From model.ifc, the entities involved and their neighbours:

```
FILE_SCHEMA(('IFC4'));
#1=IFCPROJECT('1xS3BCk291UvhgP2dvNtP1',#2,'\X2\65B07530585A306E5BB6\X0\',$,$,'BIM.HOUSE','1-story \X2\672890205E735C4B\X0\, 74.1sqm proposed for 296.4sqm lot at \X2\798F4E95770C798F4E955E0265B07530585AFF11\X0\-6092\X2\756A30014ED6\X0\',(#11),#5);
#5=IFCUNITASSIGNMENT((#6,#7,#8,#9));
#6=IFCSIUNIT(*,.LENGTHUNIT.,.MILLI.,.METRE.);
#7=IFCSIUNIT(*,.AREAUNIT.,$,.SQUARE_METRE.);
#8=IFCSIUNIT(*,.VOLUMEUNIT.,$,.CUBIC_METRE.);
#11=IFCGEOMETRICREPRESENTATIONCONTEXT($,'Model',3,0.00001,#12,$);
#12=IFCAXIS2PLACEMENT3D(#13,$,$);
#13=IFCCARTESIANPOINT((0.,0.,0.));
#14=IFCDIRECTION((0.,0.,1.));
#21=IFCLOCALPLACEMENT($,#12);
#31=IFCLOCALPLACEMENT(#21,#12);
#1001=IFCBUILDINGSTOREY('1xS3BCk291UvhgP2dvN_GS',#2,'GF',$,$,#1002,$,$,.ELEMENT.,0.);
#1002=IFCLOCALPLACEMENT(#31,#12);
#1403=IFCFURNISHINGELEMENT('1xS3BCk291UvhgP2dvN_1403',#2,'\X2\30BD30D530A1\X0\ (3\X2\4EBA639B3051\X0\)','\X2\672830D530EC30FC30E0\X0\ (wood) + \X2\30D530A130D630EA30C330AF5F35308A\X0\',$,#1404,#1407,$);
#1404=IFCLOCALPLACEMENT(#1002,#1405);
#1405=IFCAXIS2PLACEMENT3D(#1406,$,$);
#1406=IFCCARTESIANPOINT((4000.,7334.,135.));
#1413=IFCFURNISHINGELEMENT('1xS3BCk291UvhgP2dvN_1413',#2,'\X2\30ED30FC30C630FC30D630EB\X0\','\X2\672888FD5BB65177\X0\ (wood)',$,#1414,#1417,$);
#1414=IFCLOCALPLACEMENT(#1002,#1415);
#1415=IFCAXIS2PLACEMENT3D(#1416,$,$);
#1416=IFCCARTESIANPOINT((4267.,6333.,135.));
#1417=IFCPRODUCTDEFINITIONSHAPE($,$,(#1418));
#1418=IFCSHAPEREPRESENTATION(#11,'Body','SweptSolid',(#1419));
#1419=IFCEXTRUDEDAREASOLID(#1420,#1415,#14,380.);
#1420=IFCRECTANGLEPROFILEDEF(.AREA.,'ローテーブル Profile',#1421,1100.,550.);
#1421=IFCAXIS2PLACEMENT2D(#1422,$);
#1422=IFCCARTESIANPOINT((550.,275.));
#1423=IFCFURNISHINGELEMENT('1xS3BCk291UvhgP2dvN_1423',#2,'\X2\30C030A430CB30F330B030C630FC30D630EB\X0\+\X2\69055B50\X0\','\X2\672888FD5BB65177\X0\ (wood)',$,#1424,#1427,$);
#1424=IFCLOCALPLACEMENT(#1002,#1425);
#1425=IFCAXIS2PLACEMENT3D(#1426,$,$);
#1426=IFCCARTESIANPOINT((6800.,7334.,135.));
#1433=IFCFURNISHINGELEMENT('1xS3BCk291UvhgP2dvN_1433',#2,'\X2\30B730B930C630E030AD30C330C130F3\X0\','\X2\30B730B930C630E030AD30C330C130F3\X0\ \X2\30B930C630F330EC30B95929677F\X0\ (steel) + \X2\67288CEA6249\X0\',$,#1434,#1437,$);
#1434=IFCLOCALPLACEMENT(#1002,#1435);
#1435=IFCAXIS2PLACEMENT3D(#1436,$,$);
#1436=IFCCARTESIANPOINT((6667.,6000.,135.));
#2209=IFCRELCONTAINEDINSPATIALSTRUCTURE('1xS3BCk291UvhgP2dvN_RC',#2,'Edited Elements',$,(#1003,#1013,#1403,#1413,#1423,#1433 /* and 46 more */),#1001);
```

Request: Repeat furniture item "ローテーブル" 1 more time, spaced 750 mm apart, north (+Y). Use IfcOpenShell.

```python
import numpy as np
import ifcopenshell
import ifcopenshell.api.geometry
import ifcopenshell.api.root
import ifcopenshell.util.element
import ifcopenshell.util.placement
import ifcopenshell.util.unit

model = ifcopenshell.open("model.ifc")
unit_scale = ifcopenshell.util.unit.calculate_unit_scale(model)


def reuse_history(source, copy):
    """copy_class also copies each property set's owner history, people and application; keep the originals."""
    for rel in copy.IsDefinedBy:
        if rel.is_a("IfcRelDefinesByProperties") and (history := rel.RelatingPropertyDefinition.OwnerHistory):
            rel.RelatingPropertyDefinition.OwnerHistory = source.OwnerHistory
            ifcopenshell.util.element.remove_deep2(model, history)


source = model.by_guid("1xS3BCk291UvhgP2dvN_1413")
base = ifcopenshell.util.placement.get_local_placement(source.ObjectPlacement)
step = np.array([0.0, 1.0, 0.0]) * 0.75 / unit_scale

for i in range(1, 2):
    copy = ifcopenshell.api.root.copy_class(model, product=source)
    copy.Representation = ifcopenshell.util.element.copy_deep(
        model, source.Representation, exclude=["IfcGeometricRepresentationContext", "IfcRepresentationMap"]
    )
    reuse_history(source, copy)
    matrix = base.copy()
    matrix[:3, 3] += i * step
    print("added at", matrix[:3, 3].round(3) + 0.0)
    ifcopenshell.api.geometry.edit_object_placement(model, product=copy, matrix=matrix, is_si=False)

model.write("model_updated.ifc")
```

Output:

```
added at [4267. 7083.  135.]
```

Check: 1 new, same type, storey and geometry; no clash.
